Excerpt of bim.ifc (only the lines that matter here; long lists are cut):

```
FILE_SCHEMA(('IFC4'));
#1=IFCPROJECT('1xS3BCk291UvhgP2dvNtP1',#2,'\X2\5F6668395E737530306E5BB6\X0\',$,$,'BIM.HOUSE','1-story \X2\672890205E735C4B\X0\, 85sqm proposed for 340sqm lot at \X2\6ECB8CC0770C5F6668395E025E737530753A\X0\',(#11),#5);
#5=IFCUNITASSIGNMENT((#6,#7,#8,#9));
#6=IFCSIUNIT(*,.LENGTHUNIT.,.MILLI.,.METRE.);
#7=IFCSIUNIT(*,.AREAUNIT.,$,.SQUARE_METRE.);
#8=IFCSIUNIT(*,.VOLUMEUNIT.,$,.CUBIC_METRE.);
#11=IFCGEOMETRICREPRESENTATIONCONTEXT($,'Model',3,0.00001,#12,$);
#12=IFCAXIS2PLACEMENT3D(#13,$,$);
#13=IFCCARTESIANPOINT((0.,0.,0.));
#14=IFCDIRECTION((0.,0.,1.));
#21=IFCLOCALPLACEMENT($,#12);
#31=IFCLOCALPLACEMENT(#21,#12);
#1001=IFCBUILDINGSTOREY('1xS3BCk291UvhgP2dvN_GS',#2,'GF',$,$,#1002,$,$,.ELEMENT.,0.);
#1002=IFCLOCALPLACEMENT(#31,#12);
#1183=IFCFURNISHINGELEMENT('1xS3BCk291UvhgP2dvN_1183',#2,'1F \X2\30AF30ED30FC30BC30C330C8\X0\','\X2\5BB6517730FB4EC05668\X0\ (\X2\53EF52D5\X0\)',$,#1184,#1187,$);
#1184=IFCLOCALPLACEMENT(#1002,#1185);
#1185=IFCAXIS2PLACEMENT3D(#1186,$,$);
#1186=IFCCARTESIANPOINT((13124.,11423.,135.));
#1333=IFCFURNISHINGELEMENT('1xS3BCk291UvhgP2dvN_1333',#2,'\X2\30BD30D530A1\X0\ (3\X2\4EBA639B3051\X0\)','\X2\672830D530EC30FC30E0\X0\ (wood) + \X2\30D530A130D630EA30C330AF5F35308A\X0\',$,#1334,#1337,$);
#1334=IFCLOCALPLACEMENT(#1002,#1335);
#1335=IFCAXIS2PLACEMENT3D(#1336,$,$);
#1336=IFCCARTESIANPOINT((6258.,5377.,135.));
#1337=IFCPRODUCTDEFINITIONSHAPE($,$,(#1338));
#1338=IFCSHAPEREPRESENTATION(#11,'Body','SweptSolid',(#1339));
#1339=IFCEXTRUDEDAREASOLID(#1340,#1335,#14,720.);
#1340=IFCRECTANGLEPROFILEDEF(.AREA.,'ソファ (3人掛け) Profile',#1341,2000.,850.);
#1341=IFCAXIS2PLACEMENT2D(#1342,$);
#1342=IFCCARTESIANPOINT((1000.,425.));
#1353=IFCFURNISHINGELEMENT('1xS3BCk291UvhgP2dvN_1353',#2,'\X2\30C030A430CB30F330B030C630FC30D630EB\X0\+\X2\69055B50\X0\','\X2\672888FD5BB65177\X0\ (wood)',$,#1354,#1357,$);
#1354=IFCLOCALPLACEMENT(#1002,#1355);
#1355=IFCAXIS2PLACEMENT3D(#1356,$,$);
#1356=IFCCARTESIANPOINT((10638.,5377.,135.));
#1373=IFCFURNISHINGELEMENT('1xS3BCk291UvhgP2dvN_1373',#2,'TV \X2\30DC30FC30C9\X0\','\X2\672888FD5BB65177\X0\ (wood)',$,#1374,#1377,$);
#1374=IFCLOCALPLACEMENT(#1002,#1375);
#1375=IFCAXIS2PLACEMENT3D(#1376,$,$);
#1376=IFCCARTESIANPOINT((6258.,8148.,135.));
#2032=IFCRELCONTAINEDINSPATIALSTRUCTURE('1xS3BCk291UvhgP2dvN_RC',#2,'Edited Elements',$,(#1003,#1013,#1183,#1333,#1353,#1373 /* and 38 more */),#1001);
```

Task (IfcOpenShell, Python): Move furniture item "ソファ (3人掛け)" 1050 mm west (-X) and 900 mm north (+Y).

```python
import ifcopenshell
import ifcopenshell.api.geometry
import ifcopenshell.util.placement

model = ifcopenshell.open("bim.ifc")

item = model.by_guid("1xS3BCk291UvhgP2dvN_1333")
matrix = ifcopenshell.util.placement.get_local_placement(item.ObjectPlacement)
matrix[0, 3] -= 1050.0
matrix[1, 3] += 900.0
ifcopenshell.api.geometry.edit_object_placement(model, product=item, matrix=matrix, is_si=False)

print(ifcopenshell.util.placement.get_local_placement(item.ObjectPlacement).round(3) + 0.0)

model.write("bim_v2.ifc")
```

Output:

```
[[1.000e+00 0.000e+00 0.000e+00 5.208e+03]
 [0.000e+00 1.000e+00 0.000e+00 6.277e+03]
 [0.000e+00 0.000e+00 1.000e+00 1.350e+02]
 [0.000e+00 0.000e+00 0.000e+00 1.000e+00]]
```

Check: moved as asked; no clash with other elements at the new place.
